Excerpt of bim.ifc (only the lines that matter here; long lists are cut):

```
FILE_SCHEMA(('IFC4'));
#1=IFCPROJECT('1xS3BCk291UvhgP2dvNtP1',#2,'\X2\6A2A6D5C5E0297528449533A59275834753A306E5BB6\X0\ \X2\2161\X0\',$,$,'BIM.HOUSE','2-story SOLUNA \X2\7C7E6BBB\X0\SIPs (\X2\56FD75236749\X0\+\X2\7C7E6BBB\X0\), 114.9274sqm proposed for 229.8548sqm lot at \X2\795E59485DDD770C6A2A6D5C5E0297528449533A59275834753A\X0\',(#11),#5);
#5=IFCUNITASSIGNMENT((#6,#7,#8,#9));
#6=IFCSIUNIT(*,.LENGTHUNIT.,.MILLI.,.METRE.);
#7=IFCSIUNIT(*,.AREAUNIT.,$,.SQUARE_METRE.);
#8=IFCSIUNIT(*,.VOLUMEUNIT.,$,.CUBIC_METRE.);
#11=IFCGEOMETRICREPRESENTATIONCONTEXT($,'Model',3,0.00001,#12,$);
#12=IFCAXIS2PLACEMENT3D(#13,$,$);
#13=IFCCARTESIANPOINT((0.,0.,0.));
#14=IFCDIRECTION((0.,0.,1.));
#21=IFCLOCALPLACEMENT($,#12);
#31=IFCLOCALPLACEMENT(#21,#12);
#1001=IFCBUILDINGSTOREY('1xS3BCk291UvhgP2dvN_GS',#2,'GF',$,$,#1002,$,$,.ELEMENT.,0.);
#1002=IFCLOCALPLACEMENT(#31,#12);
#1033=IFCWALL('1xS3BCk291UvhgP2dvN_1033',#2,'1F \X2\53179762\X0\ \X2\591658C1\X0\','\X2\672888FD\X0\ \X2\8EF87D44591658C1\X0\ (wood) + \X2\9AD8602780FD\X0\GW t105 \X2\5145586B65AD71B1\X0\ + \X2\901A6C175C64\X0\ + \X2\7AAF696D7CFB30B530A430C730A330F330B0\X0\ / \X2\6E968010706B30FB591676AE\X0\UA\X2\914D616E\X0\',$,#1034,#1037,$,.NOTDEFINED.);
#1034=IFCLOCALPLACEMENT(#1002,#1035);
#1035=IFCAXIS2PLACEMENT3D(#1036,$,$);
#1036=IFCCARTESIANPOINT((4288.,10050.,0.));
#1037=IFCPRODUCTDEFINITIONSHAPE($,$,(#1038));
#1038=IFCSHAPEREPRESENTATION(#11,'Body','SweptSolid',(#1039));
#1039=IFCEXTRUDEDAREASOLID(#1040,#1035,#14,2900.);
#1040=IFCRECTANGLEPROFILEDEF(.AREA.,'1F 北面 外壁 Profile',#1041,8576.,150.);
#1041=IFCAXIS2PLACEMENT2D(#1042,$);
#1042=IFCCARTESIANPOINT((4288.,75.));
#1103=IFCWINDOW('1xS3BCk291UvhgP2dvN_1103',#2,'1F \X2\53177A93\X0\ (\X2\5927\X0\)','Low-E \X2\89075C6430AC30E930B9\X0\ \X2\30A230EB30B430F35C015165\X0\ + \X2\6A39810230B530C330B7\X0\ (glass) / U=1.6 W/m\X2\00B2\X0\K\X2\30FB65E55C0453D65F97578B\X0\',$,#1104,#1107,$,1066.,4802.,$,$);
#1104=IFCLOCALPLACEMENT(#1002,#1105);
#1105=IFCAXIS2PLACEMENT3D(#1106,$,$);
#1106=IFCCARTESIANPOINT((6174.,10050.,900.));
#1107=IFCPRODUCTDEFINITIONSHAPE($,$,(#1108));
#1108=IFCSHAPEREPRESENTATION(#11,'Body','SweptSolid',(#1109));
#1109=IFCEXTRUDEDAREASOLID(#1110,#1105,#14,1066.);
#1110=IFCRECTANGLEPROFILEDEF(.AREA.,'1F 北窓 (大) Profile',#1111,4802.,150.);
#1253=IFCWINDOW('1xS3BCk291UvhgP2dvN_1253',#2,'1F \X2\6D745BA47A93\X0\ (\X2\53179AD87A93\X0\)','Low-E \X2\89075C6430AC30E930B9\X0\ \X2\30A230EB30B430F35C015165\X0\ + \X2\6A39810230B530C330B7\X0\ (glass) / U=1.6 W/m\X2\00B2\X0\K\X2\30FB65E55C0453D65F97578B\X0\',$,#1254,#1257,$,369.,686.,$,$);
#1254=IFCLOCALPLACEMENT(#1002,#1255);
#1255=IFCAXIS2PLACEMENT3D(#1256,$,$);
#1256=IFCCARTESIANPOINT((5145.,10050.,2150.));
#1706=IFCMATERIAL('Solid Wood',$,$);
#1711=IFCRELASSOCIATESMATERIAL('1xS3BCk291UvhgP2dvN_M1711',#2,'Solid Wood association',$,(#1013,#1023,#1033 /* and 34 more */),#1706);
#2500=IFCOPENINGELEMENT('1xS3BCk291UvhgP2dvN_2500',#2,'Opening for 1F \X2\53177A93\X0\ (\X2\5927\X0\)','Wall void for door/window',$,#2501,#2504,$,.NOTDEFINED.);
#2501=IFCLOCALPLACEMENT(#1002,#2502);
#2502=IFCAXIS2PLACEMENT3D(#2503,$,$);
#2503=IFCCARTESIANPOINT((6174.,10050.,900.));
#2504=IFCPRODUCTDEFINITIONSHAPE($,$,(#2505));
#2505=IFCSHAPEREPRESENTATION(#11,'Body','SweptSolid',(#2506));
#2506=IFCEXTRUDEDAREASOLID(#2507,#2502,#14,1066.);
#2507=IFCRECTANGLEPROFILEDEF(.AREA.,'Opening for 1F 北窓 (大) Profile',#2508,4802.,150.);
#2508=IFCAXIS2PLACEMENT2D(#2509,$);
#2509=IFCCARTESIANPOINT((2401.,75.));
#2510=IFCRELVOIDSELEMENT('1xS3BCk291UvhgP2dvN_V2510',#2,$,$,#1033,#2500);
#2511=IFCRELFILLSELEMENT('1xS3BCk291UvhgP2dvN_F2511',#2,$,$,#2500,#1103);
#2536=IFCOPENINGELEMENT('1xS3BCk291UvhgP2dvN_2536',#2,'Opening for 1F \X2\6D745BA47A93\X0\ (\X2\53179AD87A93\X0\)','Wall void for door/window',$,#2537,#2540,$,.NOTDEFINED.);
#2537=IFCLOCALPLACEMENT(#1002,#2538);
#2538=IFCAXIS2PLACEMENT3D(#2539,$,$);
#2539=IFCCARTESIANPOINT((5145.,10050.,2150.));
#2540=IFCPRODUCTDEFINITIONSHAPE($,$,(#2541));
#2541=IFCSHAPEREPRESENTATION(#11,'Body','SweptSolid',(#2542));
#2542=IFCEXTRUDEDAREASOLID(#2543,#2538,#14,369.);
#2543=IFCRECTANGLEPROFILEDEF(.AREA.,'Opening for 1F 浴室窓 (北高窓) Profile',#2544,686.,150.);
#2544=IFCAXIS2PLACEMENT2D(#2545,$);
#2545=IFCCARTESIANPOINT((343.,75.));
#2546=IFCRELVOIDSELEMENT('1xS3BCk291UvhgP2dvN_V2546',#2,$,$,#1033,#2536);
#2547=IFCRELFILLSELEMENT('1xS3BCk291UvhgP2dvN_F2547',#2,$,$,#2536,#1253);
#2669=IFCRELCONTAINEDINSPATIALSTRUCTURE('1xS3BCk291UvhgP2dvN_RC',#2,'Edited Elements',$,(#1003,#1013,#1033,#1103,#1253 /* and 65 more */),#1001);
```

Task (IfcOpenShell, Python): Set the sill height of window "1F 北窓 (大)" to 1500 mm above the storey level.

```python
import numpy as np
import ifcopenshell
import ifcopenshell.api.geometry
import ifcopenshell.geom
import ifcopenshell.util.element
import ifcopenshell.util.placement
import ifcopenshell.util.shape
import ifcopenshell.util.unit

model = ifcopenshell.open("bim.ifc")
unit_scale = ifcopenshell.util.unit.calculate_unit_scale(model)

window = model.by_id(1103)
opening = window.FillsVoids[0].RelatingOpeningElement
storey = ifcopenshell.util.element.get_container(window, ifc_class="IfcBuildingStorey")
level = ifcopenshell.util.placement.get_local_placement(storey.ObjectPlacement)[2, 3]

# The opening's origin need not be at the sill, so measure its lowest point.
shape = ifcopenshell.geom.create_shape(ifcopenshell.geom.settings(), opening)
bottom = ifcopenshell.util.shape.get_shape_bottom_elevation(shape, shape.geometry) / unit_scale
dz = level + 1.5 / unit_scale - bottom

shift = np.array([0.0, 0.0, dz])
# The window is not placed relative to its opening, so move both.
for product in (opening, window):
    matrix = ifcopenshell.util.placement.get_local_placement(product.ObjectPlacement)
    matrix[:3, 3] += shift
    ifcopenshell.api.geometry.edit_object_placement(model, product=product, matrix=matrix, is_si=False)

print(f"moved by {dz * unit_scale:+.3f} m")

model.write("bim_edited.ifc")
```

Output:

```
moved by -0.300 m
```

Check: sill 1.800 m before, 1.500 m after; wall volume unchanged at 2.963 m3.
